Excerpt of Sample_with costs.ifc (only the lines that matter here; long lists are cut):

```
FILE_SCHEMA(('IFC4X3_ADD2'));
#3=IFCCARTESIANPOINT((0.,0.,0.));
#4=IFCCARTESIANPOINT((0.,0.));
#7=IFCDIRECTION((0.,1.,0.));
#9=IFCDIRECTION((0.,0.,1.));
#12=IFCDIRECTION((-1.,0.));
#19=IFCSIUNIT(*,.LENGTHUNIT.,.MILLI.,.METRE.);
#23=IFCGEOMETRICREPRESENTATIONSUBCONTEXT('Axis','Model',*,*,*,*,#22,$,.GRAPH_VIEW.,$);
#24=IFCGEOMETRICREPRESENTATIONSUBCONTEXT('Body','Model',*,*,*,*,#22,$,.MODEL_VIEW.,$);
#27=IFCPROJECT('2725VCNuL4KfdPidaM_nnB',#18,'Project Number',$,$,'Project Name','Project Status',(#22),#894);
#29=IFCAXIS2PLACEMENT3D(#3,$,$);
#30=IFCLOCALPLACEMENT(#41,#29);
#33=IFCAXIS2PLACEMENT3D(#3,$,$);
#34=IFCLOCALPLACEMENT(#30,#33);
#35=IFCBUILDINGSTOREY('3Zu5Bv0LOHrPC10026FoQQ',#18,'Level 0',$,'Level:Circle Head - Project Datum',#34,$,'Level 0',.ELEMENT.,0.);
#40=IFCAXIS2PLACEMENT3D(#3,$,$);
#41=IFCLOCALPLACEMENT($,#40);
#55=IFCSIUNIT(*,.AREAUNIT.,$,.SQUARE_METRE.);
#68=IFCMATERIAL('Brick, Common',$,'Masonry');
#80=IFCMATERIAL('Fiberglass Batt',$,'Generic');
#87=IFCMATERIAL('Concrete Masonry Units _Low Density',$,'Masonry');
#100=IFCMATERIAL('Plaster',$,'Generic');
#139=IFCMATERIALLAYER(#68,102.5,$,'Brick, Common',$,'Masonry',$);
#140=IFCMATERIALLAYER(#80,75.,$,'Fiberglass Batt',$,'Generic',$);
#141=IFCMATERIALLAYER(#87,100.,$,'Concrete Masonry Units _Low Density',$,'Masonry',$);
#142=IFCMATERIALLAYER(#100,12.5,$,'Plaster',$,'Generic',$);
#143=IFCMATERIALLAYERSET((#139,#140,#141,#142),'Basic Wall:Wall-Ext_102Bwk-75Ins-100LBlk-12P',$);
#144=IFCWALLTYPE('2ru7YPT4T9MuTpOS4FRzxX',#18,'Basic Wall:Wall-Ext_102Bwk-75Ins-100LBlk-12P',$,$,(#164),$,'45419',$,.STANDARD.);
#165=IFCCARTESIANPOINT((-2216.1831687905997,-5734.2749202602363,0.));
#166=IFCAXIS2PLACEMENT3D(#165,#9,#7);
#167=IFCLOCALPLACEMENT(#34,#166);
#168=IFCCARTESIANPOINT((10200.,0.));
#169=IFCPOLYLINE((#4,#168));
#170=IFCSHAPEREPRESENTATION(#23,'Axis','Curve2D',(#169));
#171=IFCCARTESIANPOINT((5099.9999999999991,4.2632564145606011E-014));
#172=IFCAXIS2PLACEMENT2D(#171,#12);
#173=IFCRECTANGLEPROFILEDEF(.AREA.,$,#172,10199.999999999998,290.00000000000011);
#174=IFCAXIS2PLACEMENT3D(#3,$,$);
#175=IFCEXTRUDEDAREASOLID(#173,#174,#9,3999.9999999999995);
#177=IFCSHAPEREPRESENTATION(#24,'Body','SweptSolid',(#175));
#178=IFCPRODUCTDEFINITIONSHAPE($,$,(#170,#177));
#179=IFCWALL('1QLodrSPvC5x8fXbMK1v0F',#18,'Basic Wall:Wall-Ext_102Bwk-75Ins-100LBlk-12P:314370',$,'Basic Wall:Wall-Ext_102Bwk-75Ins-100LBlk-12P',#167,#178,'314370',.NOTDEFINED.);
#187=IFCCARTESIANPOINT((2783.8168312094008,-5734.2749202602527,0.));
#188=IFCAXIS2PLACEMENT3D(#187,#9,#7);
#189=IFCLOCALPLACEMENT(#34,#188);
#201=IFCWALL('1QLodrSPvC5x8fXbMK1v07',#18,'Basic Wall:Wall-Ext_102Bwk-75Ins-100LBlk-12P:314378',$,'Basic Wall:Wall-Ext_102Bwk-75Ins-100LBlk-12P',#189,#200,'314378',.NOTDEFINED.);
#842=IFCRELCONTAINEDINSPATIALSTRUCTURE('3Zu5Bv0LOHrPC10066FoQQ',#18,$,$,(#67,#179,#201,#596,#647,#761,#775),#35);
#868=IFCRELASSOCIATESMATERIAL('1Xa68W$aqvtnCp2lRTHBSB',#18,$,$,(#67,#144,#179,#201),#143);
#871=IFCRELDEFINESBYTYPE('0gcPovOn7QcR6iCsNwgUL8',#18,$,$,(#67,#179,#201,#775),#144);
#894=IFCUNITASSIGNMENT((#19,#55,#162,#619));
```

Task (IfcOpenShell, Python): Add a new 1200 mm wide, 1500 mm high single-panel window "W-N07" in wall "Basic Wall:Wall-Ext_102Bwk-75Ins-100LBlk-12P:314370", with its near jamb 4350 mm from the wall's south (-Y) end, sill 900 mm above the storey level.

```python
import numpy as np
import ifcopenshell
import ifcopenshell.api.feature
import ifcopenshell.api.geometry
import ifcopenshell.api.root
import ifcopenshell.api.spatial
import ifcopenshell.geom
import ifcopenshell.util.element
import ifcopenshell.util.placement
import ifcopenshell.util.representation
import ifcopenshell.util.shape
import ifcopenshell.util.unit

model = ifcopenshell.open("Sample_with costs.ifc")
unit_scale = ifcopenshell.util.unit.calculate_unit_scale(model)
settings = ifcopenshell.geom.settings()


def volume(element):
    """Net volume in cubic metres, openings subtracted."""
    shape = ifcopenshell.geom.create_shape(settings, element)
    return ifcopenshell.util.shape.get_volume(shape.geometry)


wall = model.by_guid("1QLodrSPvC5x8fXbMK1v0F")
storey = ifcopenshell.util.element.get_container(wall, ifc_class="IfcBuildingStorey")
context = ifcopenshell.util.representation.get_context(model, "Model", "Body", "MODEL_VIEW")
before = volume(wall)

width, height, from_end, sill = 1.2, 1.5, 4.35, 0.9  # metres

# The wall runs along its own X axis, and the end named is its -X end.
wall_shape = ifcopenshell.geom.create_shape(settings, wall)
x, y, z = ifcopenshell.util.shape.get_vertices(wall_shape.geometry).T
start = x.min() + from_end
face, thickness = float(y.min()), float(y.max() - y.min())
wall_matrix = ifcopenshell.util.placement.get_local_placement(wall.ObjectPlacement)
level = ifcopenshell.util.placement.get_local_placement(storey.ObjectPlacement)[2, 3]


def in_wall(x, y):
    """Placement at x, y metres in the wall's axes, at sill height."""
    matrix = wall_matrix.copy()
    matrix[:, 3] = wall_matrix @ np.array([x / unit_scale, y / unit_scale, 0.0, 1.0])
    matrix[2, 3] = level + sill / unit_scale
    return matrix


# Opening: a box that overshoots both wall faces by 50 mm.
opening = ifcopenshell.api.root.create_entity(model, ifc_class="IfcOpeningElement", predefined_type="OPENING")
box = ifcopenshell.api.geometry.add_wall_representation(
    model, context=context, length=width, height=height, thickness=thickness + 0.1
)
ifcopenshell.api.geometry.assign_representation(model, product=opening, representation=box)
ifcopenshell.api.geometry.edit_object_placement(model, product=opening, matrix=in_wall(start, face - 0.05), is_si=False)
ifcopenshell.api.feature.add_feature(model, feature=opening, element=wall)

window = ifcopenshell.api.root.create_entity(model, ifc_class="IfcWindow", name="W-N07", predefined_type="WINDOW")
window.OverallWidth, window.OverallHeight = width / unit_scale, height / unit_scale
window.PartitioningType = "SINGLE_PANEL"
body = ifcopenshell.api.geometry.add_window_representation(
    model,
    context=context,
    overall_width=window.OverallWidth,
    overall_height=window.OverallHeight,
    partition_type="SINGLE_PANEL",
)
ifcopenshell.api.geometry.assign_representation(model, product=window, representation=body)
ifcopenshell.api.spatial.assign_container(model, products=[window], relating_structure=storey)
ifcopenshell.api.feature.add_filling(model, opening=opening, element=window)

# Centre the window in the wall's thickness.
ifcopenshell.api.geometry.edit_object_placement(model, product=window, matrix=in_wall(start, face), is_si=False)
window_shape = ifcopenshell.geom.create_shape(settings, window)
depth = ifcopenshell.util.shape.get_vertices(window_shape.geometry)[:, 1]
offset = face + thickness / 2 - (depth.min() + depth.max()) / 2
ifcopenshell.api.geometry.edit_object_placement(model, product=window, matrix=in_wall(start, offset), is_si=False)

after = volume(wall)

print(f"wall volume {before:.3f} -> {after:.3f} m3")

model.write("Sample_with costs_edited.ifc")
```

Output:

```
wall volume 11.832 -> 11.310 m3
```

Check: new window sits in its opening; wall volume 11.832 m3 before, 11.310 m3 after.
